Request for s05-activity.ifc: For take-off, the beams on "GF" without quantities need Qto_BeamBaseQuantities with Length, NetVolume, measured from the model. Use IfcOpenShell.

First a look at what the model holds.

```python
import ifcopenshell
import ifcopenshell.util.element
import ifcopenshell.util.unit

model = ifcopenshell.open("s05-activity.ifc")
print(model.schema)
for unit_type in ("LENGTHUNIT", "AREAUNIT", "VOLUMEUNIT"):
    print(unit_type, ifcopenshell.util.unit.calculate_unit_scale(model, unit_type))
storey = next(s for s in model.by_type("IfcBuildingStorey") if s.Name == "GF")
beams = [e for e in ifcopenshell.util.element.get_decomposition(storey) if e.is_a("IfcBeam")]
for e in sorted(beams, key=lambda e: e.id()):
    print(e.id(), e.is_a(), e.Name, list(ifcopenshell.util.element.get_psets(e, qtos_only=True)), sep=" | ")
```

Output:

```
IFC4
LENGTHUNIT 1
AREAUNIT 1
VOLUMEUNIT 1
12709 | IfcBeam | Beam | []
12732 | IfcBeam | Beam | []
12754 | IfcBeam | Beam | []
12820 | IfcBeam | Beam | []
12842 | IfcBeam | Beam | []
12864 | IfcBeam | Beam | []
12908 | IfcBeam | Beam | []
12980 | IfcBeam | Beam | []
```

```python
import ifcopenshell
import ifcopenshell.api.pset
import ifcopenshell.geom
import ifcopenshell.util.element
import ifcopenshell.util.shape
import ifcopenshell.util.unit

model = ifcopenshell.open("s05-activity.ifc")
unit_scale = ifcopenshell.util.unit.calculate_unit_scale(model)
volume_scale = ifcopenshell.util.unit.calculate_unit_scale(model, "VOLUMEUNIT")
settings = ifcopenshell.geom.settings()

storey = next(s for s in model.by_type("IfcBuildingStorey") if s.Name == "GF")
beams = [e for e in ifcopenshell.util.element.get_decomposition(storey) if e.is_a("IfcBeam")]

for e in sorted(beams, key=lambda e: e.id()):
    if ifcopenshell.util.element.get_psets(e, qtos_only=True, should_inherit=False):
        continue
    # Geometry comes back in metres, in the element's own axes.
    shape = ifcopenshell.geom.create_shape(settings, e)
    values = {
        "Length": ifcopenshell.util.shape.get_max_xyz(shape.geometry) / unit_scale,
        "NetVolume": ifcopenshell.util.shape.get_volume(shape.geometry) / volume_scale,
    }
    qto = ifcopenshell.api.pset.add_qto(model, product=e, name="Qto_BeamBaseQuantities")
    ifcopenshell.api.pset.edit_qto(model, qto=qto, properties=values)
    print(e.id(), {k: round(v, 3) for k, v in values.items()})

model.write("s05-activity_rev.ifc")
```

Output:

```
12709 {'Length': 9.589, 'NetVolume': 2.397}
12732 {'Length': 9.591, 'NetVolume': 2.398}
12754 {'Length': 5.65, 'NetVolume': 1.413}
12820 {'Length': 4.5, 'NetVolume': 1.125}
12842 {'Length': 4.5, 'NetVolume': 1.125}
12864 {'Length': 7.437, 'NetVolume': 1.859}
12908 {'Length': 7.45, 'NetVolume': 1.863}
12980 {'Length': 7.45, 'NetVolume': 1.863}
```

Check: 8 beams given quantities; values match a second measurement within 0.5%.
